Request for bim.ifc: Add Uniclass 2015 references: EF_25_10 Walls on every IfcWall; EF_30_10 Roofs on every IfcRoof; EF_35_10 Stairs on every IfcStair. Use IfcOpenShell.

First a look at what the model holds.

```python
import ifcopenshell

model = ifcopenshell.open("bim.ifc")
print(model.schema)
print("classifications:", [c.Name for c in model.by_type("IfcClassification")])
for ifc_class in ("IfcDoor", "IfcRoof", "IfcStair", "IfcWall", "IfcWindow"):
    print(ifc_class, len(model.by_type(ifc_class)))
```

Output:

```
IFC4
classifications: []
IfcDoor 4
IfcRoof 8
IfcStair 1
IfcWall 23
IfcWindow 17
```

```python
import ifcopenshell
import ifcopenshell.api.classification

model = ifcopenshell.open("bim.ifc")

system = ifcopenshell.api.classification.add_classification(model, classification="Uniclass 2015")

codes = {
    "IfcWall": ("EF_25_10", "Walls"),
    "IfcRoof": ("EF_30_10", "Roofs"),
    "IfcStair": ("EF_35_10", "Stairs"),
}
for ifc_class, (code, name) in codes.items():
    products = model.by_type(ifc_class)
    ifcopenshell.api.classification.add_reference(
        model, products=products, classification=system, identification=code, name=name
    )
    print(code, len(products))

model.write("bim_rev.ifc")
```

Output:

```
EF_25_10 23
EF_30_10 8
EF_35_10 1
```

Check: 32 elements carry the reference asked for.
